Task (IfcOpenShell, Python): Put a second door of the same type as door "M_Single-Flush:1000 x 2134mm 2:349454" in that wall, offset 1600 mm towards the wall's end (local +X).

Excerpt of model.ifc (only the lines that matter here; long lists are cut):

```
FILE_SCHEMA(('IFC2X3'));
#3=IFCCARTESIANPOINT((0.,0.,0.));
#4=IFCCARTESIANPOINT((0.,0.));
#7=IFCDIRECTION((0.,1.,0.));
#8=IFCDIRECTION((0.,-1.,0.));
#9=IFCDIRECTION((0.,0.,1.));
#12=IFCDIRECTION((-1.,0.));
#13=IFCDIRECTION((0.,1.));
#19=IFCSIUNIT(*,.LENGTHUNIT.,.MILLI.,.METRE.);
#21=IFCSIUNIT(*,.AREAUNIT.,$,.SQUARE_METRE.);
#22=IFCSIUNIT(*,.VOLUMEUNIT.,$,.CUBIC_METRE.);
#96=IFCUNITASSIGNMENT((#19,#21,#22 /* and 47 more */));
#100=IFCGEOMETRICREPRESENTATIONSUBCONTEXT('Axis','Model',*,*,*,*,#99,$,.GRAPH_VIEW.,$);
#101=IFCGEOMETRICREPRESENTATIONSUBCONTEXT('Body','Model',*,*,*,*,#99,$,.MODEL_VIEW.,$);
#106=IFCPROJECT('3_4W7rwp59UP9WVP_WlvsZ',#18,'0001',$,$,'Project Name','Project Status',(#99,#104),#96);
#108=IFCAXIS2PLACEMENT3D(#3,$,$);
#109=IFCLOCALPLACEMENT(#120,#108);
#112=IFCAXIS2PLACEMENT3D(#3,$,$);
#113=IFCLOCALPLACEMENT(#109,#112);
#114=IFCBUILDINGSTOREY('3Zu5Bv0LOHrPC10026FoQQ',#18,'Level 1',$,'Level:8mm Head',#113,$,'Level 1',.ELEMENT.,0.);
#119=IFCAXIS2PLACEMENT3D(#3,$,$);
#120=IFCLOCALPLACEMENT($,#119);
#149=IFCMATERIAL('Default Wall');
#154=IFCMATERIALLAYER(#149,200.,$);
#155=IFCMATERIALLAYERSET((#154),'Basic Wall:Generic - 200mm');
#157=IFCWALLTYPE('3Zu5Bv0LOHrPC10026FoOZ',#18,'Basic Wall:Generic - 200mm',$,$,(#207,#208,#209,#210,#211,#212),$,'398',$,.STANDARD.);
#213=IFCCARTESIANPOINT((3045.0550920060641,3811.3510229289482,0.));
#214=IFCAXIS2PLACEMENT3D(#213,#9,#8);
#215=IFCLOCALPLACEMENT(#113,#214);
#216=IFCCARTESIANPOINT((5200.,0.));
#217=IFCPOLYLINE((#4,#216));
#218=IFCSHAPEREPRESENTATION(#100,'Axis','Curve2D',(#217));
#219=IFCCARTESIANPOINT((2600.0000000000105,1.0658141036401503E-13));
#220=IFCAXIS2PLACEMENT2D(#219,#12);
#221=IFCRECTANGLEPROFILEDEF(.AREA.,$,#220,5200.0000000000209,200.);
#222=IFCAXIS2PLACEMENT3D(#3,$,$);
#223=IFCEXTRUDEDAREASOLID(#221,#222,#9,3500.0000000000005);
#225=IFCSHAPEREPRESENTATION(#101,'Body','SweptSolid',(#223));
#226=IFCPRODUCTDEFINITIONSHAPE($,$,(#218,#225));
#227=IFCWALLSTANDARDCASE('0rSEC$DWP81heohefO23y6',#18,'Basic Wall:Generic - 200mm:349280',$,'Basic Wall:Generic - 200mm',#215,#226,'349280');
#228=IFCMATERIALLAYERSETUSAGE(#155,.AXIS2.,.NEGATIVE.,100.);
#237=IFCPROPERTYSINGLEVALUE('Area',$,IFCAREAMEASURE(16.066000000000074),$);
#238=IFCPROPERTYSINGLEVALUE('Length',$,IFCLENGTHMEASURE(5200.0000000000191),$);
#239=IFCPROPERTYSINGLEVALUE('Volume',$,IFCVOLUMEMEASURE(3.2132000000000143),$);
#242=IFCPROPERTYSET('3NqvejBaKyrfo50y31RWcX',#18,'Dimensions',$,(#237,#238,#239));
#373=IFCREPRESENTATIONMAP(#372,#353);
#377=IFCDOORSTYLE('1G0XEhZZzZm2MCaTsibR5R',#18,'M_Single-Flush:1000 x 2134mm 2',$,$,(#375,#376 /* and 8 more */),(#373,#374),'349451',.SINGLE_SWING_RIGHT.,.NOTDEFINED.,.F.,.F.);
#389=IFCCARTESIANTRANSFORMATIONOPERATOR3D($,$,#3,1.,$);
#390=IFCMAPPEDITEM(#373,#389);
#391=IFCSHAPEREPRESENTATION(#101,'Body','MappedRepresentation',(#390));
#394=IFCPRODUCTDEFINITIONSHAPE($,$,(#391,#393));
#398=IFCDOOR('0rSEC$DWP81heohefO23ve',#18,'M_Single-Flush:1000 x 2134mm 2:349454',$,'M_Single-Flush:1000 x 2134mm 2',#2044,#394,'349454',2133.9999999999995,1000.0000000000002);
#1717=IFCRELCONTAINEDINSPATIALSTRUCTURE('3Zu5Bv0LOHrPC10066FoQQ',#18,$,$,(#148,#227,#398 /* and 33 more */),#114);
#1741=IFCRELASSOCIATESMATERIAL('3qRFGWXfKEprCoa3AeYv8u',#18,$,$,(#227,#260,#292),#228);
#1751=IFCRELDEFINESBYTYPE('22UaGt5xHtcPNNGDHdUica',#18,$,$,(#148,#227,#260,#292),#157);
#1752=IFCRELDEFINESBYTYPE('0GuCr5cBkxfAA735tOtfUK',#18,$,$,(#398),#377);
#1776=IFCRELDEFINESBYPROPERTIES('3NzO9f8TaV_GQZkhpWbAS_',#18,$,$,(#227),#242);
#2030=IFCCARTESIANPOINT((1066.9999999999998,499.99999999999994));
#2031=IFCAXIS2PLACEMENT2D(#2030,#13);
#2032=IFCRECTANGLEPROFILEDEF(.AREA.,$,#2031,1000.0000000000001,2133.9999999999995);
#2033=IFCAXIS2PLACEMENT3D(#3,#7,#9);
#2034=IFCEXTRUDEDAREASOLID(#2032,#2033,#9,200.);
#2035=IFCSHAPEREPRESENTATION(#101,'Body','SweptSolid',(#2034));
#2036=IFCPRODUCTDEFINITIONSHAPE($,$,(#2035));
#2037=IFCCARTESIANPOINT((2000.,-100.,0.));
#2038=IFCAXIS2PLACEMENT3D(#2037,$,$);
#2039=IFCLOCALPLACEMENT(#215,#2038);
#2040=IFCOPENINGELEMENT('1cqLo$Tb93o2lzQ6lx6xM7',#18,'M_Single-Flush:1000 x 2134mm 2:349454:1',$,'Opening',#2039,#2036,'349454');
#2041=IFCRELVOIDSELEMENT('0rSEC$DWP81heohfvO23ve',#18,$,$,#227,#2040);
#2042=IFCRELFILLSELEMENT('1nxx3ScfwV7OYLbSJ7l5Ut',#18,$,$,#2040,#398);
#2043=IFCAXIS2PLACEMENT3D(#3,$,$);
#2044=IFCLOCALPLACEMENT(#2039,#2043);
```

```python
import ifcopenshell
import ifcopenshell.api.feature
import ifcopenshell.api.geometry
import ifcopenshell.api.pset
import ifcopenshell.api.root
import ifcopenshell.geom
import ifcopenshell.util.element
import ifcopenshell.util.placement
import ifcopenshell.util.shape
import ifcopenshell.util.unit

model = ifcopenshell.open("model.ifc")
unit_scale = ifcopenshell.util.unit.calculate_unit_scale(model)
area_scale = ifcopenshell.util.unit.calculate_unit_scale(model, "AREAUNIT")
volume_scale = ifcopenshell.util.unit.calculate_unit_scale(model, "VOLUMEUNIT")
settings = ifcopenshell.geom.settings()


def volume(element):
    """Net volume in cubic metres, openings subtracted."""
    shape = ifcopenshell.geom.create_shape(settings, element)
    return ifcopenshell.util.shape.get_volume(shape.geometry)


def reuse_history(source, copy):
    """copy_class also copies each property set's owner history, people and application; keep the originals."""
    for rel in copy.IsDefinedBy:
        if rel.is_a("IfcRelDefinesByProperties") and (history := rel.RelatingPropertyDefinition.OwnerHistory):
            rel.RelatingPropertyDefinition.OwnerHistory = source.OwnerHistory
            ifcopenshell.util.element.remove_deep2(model, history)


door = model.by_guid("0rSEC$DWP81heohefO23ve")
opening = door.FillsVoids[0].RelatingOpeningElement
wall = opening.VoidsElements[0].RelatingBuildingElement
before = volume(wall)
shift = ifcopenshell.util.placement.get_local_placement(wall.ObjectPlacement)[:3, 0] * 1.6 / unit_scale

# copy_class copies the void relationship, type, container and properties, but no geometry.
new_opening = ifcopenshell.api.root.copy_class(model, product=opening)
new_opening.Representation = ifcopenshell.util.element.copy_deep(
    model, opening.Representation, exclude=["IfcGeometricRepresentationContext", "IfcRepresentationMap"]
)
new_opening.Name = "M_Single-Flush:1000 x 2134mm 2"
new_opening.Tag = None
new_door = ifcopenshell.api.root.copy_class(model, product=door)
new_door.Representation = ifcopenshell.util.element.copy_deep(
    model, door.Representation, exclude=["IfcGeometricRepresentationContext", "IfcRepresentationMap"]
)
new_door.Name = "M_Single-Flush:1000 x 2134mm 2"
new_door.Tag = None
reuse_history(door, new_door)
fills = ifcopenshell.api.feature.add_filling(model, opening=new_opening, element=new_door)
fills.OwnerHistory = new_door.OwnerHistory  # required in IFC2X3

for old, new in ((opening, new_opening), (door, new_door)):
    matrix = ifcopenshell.util.placement.get_local_placement(old.ObjectPlacement)
    matrix[:3, 3] += shift
    ifcopenshell.api.geometry.edit_object_placement(model, product=new, matrix=matrix, is_si=False)

after = volume(wall)
thickness = 0.2  # wall thickness in metres

# Update the wall's stored quantities.
pset = model.by_id(ifcopenshell.util.element.get_pset(wall, "Dimensions", should_inherit=False)["id"])
ifcopenshell.api.pset.edit_pset(model, pset=pset, properties={
    "Area": model.create_entity("IfcAreaMeasure", after / thickness / area_scale),
    "Volume": model.create_entity("IfcVolumeMeasure", after / volume_scale),
})

print(f"wall volume {before:.3f} -> {after:.3f} m3")

model.write("model-out.ifc")
```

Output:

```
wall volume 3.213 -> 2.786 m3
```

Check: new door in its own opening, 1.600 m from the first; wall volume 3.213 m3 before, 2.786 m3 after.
